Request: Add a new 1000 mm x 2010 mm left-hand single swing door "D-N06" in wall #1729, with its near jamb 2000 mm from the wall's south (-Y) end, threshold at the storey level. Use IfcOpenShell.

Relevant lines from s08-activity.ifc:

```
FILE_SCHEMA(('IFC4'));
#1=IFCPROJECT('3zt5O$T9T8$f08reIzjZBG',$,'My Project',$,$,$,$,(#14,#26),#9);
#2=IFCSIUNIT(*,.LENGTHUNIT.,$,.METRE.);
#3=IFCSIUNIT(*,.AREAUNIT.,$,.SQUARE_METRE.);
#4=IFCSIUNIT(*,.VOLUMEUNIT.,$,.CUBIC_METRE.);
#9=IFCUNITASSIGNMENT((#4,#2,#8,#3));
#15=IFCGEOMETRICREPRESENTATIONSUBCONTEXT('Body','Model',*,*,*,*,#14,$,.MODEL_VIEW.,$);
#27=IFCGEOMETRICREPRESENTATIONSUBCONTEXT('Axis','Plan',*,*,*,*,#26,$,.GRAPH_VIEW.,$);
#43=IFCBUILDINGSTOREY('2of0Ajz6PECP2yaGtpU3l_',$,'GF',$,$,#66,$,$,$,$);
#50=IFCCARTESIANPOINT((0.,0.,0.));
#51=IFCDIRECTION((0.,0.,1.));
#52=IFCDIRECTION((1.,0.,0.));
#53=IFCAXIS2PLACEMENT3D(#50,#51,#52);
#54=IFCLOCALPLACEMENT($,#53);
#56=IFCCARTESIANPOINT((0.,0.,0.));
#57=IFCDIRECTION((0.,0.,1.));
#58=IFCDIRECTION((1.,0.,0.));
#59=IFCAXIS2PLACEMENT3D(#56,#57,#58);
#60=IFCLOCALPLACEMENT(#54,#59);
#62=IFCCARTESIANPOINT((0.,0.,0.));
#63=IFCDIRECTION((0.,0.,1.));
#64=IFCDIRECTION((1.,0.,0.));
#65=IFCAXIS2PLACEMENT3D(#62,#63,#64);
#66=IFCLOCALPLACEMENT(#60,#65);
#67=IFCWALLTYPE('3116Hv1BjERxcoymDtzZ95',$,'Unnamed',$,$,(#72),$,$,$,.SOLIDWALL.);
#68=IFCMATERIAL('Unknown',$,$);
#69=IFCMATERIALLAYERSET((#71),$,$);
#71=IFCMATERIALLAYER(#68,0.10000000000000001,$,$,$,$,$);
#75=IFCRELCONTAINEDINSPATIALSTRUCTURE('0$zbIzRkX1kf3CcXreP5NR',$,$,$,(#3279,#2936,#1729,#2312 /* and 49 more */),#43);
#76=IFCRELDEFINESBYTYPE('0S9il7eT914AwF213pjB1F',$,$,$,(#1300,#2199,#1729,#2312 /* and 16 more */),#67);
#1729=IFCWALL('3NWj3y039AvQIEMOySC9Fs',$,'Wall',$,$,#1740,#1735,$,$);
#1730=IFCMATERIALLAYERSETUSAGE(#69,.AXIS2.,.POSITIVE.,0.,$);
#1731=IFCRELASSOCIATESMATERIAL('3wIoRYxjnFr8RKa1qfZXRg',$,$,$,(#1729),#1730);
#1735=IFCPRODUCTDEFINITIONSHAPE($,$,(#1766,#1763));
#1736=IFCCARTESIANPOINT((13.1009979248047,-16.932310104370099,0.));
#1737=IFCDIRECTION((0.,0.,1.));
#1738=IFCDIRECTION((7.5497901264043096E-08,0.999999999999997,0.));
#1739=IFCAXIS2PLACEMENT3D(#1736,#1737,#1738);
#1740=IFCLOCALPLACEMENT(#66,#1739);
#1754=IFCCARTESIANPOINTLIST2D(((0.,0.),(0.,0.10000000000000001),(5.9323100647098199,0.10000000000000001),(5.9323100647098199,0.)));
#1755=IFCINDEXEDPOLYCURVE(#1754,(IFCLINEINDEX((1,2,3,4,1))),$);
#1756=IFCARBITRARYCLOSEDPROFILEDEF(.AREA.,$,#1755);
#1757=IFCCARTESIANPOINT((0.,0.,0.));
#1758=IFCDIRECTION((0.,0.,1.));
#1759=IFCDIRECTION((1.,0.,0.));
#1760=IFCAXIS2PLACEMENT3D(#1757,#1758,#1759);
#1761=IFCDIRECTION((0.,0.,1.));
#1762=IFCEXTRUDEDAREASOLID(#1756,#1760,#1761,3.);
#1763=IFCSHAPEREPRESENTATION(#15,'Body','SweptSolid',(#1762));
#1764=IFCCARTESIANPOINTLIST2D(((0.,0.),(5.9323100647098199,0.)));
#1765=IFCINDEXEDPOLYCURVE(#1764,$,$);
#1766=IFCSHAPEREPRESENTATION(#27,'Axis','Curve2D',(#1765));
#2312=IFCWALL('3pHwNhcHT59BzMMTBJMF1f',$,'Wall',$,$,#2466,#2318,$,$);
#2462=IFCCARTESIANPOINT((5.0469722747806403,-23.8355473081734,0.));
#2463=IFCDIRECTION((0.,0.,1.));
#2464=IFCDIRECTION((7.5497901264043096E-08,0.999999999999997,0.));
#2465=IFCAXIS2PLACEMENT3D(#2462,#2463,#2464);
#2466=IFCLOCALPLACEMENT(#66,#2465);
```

```python
import numpy as np
import ifcopenshell
import ifcopenshell.api.feature
import ifcopenshell.api.geometry
import ifcopenshell.api.root
import ifcopenshell.api.spatial
import ifcopenshell.geom
import ifcopenshell.util.element
import ifcopenshell.util.placement
import ifcopenshell.util.representation
import ifcopenshell.util.shape
import ifcopenshell.util.unit

model = ifcopenshell.open("s08-activity.ifc")
unit_scale = ifcopenshell.util.unit.calculate_unit_scale(model)
settings = ifcopenshell.geom.settings()


def volume(element):
    """Net volume in cubic metres, openings subtracted."""
    shape = ifcopenshell.geom.create_shape(settings, element)
    return ifcopenshell.util.shape.get_volume(shape.geometry)


wall = model.by_id(1729)
storey = ifcopenshell.util.element.get_container(wall, ifc_class="IfcBuildingStorey")
context = ifcopenshell.util.representation.get_context(model, "Model", "Body", "MODEL_VIEW")
before = volume(wall)

width, height, from_end, sill = 1, 2.01, 2, 0.0  # metres

# The wall runs along its own X axis, and the end named is its -X end.
wall_shape = ifcopenshell.geom.create_shape(settings, wall)
x, y, z = ifcopenshell.util.shape.get_vertices(wall_shape.geometry).T
start = x.min() + from_end
face, thickness = float(y.min()), float(y.max() - y.min())
wall_matrix = ifcopenshell.util.placement.get_local_placement(wall.ObjectPlacement)
level = ifcopenshell.util.placement.get_local_placement(storey.ObjectPlacement)[2, 3]


def in_wall(x, y):
    """Placement at x, y metres in the wall's axes, at sill height."""
    matrix = wall_matrix.copy()
    matrix[:, 3] = wall_matrix @ np.array([x / unit_scale, y / unit_scale, 0.0, 1.0])
    matrix[2, 3] = level + sill / unit_scale
    return matrix


# Opening: a box that overshoots both wall faces by 50 mm.
opening = ifcopenshell.api.root.create_entity(model, ifc_class="IfcOpeningElement", predefined_type="OPENING")
box = ifcopenshell.api.geometry.add_wall_representation(
    model, context=context, length=width, height=height, thickness=thickness + 0.1
)
ifcopenshell.api.geometry.assign_representation(model, product=opening, representation=box)
ifcopenshell.api.geometry.edit_object_placement(model, product=opening, matrix=in_wall(start, face - 0.05), is_si=False)
ifcopenshell.api.feature.add_feature(model, feature=opening, element=wall)

door = ifcopenshell.api.root.create_entity(model, ifc_class="IfcDoor", name="D-N06", predefined_type="DOOR")
door.OverallWidth, door.OverallHeight = width / unit_scale, height / unit_scale
door.OperationType = "SINGLE_SWING_LEFT"
body = ifcopenshell.api.geometry.add_door_representation(
    model,
    context=context,
    overall_width=door.OverallWidth,
    overall_height=door.OverallHeight,
    operation_type="SINGLE_SWING_LEFT",
    lining_properties={"LiningDepth": thickness / unit_scale, "ThresholdDepth": thickness / unit_scale},
)
ifcopenshell.api.geometry.assign_representation(model, product=door, representation=body)
ifcopenshell.api.spatial.assign_container(model, products=[door], relating_structure=storey)
ifcopenshell.api.feature.add_filling(model, opening=opening, element=door)

# The lining spans the wall, so the door starts at the wall face.
ifcopenshell.api.geometry.edit_object_placement(model, product=door, matrix=in_wall(start, face), is_si=False)

after = volume(wall)

print(f"wall volume {before:.3f} -> {after:.3f} m3")

model.write("s08-activity_edited.ifc")
```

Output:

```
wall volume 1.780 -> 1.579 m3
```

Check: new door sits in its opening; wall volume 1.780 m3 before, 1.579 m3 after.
